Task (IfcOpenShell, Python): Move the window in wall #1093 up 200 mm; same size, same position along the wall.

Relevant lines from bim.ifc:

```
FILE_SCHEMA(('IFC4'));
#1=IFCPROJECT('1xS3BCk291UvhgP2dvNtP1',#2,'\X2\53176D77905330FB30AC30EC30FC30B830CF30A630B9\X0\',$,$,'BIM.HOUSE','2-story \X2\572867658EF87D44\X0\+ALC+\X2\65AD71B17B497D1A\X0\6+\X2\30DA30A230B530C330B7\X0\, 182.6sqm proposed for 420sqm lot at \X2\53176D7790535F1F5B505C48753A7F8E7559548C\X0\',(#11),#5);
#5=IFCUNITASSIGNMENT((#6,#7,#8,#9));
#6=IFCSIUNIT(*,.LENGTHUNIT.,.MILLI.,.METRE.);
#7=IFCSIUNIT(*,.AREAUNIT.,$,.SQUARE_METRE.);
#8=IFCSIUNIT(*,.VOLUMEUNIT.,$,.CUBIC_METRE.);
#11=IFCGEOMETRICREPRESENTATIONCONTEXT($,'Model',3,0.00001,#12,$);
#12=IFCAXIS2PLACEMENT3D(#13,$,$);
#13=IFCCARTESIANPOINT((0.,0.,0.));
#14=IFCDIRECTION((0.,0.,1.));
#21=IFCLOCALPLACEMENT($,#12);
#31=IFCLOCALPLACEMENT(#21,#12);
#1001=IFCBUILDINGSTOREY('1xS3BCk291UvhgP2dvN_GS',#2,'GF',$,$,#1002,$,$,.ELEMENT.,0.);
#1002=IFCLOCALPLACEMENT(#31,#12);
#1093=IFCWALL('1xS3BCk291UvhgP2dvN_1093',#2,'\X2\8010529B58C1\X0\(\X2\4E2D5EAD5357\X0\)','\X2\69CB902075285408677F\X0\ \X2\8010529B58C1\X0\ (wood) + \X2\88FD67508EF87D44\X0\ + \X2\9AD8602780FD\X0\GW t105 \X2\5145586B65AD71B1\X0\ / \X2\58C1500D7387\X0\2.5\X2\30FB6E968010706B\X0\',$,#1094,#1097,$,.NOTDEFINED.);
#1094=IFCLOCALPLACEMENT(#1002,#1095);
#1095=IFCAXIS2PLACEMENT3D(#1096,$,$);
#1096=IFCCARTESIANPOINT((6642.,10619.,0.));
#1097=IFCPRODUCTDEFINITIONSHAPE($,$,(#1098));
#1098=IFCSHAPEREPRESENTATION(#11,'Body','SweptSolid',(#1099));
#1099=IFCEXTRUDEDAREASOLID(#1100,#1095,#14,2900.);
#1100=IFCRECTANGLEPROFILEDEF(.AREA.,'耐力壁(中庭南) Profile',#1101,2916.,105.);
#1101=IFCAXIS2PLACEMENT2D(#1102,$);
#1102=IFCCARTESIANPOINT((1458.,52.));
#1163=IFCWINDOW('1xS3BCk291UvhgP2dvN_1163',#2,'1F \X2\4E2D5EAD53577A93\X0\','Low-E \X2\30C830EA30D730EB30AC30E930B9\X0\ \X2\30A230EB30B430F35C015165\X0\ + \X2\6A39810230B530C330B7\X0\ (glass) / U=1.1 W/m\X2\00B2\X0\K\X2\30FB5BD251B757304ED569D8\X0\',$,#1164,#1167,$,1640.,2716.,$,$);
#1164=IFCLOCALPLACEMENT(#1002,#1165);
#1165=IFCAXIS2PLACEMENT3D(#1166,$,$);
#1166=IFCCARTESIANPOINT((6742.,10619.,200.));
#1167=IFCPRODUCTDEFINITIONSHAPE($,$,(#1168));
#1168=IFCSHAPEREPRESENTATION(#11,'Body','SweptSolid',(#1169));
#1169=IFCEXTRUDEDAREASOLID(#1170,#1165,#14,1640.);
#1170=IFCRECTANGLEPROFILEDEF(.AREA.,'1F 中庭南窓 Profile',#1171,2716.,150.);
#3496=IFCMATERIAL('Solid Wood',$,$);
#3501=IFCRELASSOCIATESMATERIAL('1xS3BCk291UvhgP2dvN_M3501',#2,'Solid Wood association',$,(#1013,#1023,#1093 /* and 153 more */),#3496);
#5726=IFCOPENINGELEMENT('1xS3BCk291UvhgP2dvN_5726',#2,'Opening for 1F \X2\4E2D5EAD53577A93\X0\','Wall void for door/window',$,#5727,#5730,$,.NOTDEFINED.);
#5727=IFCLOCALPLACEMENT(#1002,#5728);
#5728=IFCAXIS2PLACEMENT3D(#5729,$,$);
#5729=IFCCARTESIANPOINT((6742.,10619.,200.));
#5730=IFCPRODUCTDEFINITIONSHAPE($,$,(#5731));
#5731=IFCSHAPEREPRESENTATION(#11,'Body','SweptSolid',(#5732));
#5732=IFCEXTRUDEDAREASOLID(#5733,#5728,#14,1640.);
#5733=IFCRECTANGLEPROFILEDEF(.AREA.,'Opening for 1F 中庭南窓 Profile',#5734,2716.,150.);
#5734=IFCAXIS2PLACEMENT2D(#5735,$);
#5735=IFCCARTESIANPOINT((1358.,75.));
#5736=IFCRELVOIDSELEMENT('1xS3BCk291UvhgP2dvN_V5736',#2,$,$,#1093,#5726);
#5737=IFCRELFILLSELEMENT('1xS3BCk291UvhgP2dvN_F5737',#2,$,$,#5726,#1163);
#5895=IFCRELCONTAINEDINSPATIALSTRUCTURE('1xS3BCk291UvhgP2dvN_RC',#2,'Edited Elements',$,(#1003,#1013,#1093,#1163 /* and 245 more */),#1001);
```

```python
import numpy as np
import ifcopenshell
import ifcopenshell.api.geometry
import ifcopenshell.util.placement
import ifcopenshell.util.unit

model = ifcopenshell.open("bim.ifc")
unit_scale = ifcopenshell.util.unit.calculate_unit_scale(model)

window = model.by_id(1163)
opening = window.FillsVoids[0].RelatingOpeningElement
dz = 0.2 / unit_scale

shift = np.array([0.0, 0.0, dz])
# The window is not placed relative to its opening, so move both.
for product in (opening, window):
    matrix = ifcopenshell.util.placement.get_local_placement(product.ObjectPlacement)
    matrix[:3, 3] += shift
    ifcopenshell.api.geometry.edit_object_placement(model, product=product, matrix=matrix, is_si=False)

print(f"moved by {dz * unit_scale:+.3f} m")

model.write("bim_rev.ifc")
```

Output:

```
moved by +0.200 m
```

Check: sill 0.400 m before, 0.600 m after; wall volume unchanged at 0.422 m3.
